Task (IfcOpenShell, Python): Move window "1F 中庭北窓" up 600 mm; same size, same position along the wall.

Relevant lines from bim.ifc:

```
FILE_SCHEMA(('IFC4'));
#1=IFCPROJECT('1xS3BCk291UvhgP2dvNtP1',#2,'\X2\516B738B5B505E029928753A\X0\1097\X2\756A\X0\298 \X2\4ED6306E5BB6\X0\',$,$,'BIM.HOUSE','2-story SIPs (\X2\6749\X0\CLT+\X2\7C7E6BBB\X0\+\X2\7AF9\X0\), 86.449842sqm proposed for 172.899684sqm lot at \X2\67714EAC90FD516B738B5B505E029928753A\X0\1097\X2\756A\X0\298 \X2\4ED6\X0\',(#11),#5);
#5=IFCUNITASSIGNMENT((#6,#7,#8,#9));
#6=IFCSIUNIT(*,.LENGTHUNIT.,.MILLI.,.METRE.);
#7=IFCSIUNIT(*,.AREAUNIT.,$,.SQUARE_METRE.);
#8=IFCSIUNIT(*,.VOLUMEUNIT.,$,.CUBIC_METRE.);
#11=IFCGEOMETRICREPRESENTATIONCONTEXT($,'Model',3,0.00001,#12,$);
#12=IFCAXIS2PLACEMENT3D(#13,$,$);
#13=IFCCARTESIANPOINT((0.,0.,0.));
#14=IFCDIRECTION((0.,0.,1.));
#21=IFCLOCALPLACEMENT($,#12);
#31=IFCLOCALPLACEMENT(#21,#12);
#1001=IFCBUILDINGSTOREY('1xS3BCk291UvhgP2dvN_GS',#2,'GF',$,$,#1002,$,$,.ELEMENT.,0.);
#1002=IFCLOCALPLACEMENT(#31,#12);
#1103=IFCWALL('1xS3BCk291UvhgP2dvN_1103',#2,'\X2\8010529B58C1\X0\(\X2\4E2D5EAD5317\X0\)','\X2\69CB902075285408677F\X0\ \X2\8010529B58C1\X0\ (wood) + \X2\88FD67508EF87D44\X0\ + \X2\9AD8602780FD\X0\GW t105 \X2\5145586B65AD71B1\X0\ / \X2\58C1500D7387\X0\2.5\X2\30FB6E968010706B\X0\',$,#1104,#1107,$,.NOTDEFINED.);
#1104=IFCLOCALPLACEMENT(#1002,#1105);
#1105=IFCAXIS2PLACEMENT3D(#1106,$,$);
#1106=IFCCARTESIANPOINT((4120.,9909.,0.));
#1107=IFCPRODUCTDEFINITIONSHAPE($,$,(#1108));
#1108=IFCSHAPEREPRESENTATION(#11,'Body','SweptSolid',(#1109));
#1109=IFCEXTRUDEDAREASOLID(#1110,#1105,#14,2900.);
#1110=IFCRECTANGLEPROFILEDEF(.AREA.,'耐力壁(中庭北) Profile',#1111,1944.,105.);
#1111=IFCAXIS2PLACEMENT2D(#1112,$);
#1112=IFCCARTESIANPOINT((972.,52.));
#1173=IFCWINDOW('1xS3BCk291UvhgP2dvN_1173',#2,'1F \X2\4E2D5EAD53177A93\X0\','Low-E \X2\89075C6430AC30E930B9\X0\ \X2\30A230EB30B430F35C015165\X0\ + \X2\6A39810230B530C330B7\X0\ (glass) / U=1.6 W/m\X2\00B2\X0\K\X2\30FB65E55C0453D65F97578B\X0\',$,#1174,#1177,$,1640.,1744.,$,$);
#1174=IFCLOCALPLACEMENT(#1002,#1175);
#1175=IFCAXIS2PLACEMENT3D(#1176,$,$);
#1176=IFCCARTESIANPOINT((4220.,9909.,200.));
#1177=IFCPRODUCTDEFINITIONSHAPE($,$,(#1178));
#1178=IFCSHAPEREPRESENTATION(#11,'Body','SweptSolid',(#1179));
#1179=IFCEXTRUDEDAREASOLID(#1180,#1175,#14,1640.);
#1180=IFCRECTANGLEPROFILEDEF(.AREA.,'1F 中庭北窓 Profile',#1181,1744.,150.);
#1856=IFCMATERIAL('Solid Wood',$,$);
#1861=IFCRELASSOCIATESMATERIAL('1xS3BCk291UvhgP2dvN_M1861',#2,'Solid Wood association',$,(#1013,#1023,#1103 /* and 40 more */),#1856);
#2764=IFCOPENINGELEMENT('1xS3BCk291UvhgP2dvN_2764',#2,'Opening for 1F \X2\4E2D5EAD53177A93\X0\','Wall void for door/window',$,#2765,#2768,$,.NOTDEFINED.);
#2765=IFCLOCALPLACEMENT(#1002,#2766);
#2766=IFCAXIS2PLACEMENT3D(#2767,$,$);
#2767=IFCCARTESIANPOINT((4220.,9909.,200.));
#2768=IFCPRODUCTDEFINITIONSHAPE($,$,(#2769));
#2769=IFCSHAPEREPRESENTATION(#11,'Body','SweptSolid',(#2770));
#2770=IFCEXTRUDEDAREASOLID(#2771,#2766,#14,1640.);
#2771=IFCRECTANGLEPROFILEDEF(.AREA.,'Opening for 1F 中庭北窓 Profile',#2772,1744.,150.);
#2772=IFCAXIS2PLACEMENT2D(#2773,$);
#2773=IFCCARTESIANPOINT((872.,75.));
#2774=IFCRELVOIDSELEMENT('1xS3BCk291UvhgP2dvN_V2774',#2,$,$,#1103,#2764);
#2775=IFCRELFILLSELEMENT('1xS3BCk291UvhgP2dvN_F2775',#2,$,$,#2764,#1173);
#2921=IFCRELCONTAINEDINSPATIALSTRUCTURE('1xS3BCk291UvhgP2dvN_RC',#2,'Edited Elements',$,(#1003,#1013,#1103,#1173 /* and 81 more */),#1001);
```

```python
import numpy as np
import ifcopenshell
import ifcopenshell.api.geometry
import ifcopenshell.util.placement
import ifcopenshell.util.unit

model = ifcopenshell.open("bim.ifc")
unit_scale = ifcopenshell.util.unit.calculate_unit_scale(model)

window = model.by_guid("1xS3BCk291UvhgP2dvN_1173")
opening = window.FillsVoids[0].RelatingOpeningElement
dz = 0.6 / unit_scale

shift = np.array([0.0, 0.0, dz])
# The window is not placed relative to its opening, so move both.
for product in (opening, window):
    matrix = ifcopenshell.util.placement.get_local_placement(product.ObjectPlacement)
    matrix[:3, 3] += shift
    ifcopenshell.api.geometry.edit_object_placement(model, product=product, matrix=matrix, is_si=False)

print(f"moved by {dz * unit_scale:+.3f} m")

model.write("bim_v2.ifc")
```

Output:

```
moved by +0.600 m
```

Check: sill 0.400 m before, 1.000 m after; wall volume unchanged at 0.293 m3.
